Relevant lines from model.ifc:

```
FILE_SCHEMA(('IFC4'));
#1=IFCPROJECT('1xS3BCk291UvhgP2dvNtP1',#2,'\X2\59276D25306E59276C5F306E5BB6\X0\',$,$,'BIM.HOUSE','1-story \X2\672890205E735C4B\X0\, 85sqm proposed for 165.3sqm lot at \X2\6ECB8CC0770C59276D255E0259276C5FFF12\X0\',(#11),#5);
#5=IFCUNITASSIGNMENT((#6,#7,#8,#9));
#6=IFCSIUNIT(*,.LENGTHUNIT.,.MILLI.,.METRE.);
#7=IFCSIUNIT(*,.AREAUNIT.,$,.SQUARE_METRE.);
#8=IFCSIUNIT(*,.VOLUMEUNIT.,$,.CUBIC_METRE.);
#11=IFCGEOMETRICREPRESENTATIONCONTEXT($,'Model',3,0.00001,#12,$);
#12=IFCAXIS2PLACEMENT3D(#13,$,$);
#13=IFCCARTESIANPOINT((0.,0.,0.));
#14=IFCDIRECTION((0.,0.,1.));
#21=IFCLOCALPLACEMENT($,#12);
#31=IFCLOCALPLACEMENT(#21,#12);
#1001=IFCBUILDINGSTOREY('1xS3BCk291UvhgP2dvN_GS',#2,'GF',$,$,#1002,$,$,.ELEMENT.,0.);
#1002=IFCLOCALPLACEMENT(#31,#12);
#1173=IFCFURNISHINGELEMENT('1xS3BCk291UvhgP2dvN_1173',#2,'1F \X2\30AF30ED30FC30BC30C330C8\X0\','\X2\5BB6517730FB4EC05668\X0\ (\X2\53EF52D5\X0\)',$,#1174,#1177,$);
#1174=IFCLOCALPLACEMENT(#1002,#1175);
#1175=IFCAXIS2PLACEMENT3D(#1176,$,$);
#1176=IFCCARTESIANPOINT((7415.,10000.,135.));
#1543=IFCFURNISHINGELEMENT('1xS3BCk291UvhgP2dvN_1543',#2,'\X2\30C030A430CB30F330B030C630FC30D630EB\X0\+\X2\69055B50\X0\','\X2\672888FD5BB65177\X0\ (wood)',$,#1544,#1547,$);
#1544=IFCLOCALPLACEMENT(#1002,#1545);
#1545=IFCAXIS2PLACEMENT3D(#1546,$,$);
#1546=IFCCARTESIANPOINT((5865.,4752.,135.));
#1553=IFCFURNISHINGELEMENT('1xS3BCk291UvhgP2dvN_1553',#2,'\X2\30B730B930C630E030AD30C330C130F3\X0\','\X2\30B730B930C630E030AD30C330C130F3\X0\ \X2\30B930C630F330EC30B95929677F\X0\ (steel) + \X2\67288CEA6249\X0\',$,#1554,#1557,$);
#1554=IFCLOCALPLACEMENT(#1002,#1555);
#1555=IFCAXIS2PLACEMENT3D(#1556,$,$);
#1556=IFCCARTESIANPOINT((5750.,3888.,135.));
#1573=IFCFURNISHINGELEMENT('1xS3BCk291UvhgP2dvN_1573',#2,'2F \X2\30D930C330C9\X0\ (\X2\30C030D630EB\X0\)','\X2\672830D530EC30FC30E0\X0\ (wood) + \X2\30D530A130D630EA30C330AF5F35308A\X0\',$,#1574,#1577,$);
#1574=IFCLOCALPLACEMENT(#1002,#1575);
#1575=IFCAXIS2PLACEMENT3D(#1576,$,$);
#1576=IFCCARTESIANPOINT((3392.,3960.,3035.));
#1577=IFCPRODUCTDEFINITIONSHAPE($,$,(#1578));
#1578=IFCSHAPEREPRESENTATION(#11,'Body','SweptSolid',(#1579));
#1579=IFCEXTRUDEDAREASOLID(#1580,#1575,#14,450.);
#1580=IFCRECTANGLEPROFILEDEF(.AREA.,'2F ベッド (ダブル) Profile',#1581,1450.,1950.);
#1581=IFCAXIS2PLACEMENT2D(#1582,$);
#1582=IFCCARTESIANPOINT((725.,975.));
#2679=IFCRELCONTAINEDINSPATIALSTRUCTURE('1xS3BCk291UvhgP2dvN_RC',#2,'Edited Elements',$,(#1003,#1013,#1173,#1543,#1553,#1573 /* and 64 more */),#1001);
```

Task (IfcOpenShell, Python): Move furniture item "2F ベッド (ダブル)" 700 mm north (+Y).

```python
import ifcopenshell
import ifcopenshell.api.geometry
import ifcopenshell.util.placement
import ifcopenshell.util.unit

model = ifcopenshell.open("model.ifc")
unit_scale = ifcopenshell.util.unit.calculate_unit_scale(model)

item = model.by_guid("1xS3BCk291UvhgP2dvN_1573")
matrix = ifcopenshell.util.placement.get_local_placement(item.ObjectPlacement)
matrix[1, 3] += 0.7 / unit_scale
ifcopenshell.api.geometry.edit_object_placement(model, product=item, matrix=matrix, is_si=False)

print(ifcopenshell.util.placement.get_local_placement(item.ObjectPlacement).round(3) + 0.0)

model.write("model_updated.ifc")
```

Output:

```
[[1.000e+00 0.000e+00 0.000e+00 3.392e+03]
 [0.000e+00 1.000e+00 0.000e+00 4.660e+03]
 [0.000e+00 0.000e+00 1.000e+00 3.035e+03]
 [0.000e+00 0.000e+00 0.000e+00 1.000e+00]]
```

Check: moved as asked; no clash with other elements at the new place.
